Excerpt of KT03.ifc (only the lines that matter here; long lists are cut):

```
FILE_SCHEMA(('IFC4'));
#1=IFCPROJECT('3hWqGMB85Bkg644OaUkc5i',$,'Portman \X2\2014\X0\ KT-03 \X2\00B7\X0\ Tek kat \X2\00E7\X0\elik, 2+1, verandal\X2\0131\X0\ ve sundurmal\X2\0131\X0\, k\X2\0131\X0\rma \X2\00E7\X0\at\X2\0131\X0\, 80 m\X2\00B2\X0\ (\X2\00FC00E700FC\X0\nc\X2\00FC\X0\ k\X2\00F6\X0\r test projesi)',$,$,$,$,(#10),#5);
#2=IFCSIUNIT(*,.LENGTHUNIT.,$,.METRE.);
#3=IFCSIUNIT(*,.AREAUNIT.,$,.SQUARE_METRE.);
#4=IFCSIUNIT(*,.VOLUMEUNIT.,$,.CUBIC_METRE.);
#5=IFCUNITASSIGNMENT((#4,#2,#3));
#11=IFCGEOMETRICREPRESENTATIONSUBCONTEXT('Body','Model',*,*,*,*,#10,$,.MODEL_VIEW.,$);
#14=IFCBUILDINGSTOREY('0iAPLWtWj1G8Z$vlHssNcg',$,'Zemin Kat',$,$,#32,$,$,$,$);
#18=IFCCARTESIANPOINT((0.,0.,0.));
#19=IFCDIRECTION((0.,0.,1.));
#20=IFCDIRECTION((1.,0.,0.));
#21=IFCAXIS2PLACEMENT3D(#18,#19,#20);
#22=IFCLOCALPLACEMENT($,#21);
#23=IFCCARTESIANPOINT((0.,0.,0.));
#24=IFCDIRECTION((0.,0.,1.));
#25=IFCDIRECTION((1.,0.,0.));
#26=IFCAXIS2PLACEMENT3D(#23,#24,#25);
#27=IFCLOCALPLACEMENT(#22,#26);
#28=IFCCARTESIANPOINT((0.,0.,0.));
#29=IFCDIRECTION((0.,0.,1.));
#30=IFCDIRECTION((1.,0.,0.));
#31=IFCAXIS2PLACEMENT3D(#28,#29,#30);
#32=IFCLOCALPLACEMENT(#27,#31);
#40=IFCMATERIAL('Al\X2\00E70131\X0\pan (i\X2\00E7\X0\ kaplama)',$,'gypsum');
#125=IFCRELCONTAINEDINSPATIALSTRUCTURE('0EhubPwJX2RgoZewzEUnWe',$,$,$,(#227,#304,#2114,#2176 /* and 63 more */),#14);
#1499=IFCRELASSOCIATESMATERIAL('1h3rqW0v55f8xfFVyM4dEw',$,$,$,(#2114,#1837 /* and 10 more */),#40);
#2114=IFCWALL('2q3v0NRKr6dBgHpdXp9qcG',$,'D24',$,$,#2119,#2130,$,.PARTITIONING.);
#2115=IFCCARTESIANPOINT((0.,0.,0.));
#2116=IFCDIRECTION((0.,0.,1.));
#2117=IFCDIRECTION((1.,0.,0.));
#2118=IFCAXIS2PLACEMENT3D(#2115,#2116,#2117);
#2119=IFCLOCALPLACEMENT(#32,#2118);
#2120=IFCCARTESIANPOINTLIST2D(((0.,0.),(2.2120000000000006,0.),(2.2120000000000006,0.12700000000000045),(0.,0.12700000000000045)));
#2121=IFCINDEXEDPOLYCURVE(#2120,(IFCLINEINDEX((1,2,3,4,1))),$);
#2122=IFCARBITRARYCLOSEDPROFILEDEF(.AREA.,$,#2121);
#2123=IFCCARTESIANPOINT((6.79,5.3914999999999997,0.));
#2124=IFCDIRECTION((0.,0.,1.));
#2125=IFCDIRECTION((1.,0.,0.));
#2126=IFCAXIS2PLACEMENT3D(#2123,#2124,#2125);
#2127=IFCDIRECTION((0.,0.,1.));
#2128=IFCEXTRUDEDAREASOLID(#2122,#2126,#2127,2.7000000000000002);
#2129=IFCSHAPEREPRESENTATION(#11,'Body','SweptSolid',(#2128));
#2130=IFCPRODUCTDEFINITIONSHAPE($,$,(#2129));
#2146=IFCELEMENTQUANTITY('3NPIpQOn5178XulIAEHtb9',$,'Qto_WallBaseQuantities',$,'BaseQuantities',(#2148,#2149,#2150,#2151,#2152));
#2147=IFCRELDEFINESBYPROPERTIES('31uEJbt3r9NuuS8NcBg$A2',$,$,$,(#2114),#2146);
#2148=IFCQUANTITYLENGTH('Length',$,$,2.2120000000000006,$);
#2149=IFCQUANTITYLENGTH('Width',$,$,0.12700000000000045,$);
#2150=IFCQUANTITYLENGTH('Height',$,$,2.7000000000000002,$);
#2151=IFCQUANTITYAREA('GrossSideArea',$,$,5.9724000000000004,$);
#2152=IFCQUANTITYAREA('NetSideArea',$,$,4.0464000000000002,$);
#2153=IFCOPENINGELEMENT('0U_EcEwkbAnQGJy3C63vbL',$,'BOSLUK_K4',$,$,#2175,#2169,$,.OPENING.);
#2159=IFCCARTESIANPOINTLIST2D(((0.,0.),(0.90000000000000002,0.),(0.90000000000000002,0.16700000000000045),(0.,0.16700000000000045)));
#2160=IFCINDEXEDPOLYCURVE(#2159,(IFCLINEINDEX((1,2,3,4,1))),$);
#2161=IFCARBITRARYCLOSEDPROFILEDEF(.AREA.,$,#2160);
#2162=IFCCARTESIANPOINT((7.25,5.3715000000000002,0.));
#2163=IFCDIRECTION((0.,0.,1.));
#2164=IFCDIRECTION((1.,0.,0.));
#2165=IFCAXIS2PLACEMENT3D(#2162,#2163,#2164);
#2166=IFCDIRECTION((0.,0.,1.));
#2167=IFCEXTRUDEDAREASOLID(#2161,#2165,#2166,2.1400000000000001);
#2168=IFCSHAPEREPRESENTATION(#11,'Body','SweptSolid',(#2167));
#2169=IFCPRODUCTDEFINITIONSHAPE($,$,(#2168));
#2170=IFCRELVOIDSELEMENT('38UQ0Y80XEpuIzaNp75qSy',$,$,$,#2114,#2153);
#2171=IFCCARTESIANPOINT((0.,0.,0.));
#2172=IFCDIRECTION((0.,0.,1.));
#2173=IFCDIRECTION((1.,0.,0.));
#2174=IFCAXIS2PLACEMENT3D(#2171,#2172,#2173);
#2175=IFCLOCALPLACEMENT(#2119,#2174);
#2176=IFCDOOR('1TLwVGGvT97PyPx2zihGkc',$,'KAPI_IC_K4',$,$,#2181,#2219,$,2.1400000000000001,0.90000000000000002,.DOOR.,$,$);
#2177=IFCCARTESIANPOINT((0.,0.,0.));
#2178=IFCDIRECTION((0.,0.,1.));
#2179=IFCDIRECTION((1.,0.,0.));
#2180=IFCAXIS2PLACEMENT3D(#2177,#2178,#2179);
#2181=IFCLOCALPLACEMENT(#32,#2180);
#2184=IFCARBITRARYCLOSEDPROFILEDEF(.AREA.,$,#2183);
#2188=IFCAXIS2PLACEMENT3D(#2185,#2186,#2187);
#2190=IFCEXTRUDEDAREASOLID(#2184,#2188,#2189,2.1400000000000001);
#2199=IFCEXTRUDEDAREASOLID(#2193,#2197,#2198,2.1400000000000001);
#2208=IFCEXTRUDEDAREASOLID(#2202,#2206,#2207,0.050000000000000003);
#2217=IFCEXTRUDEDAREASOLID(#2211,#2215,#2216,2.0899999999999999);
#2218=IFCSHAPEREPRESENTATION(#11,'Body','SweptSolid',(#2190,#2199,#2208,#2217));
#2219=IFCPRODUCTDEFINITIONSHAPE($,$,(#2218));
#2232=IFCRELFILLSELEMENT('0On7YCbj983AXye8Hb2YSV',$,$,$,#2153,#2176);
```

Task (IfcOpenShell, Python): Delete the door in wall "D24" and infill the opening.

```python
import ifcopenshell
import ifcopenshell.api.feature
import ifcopenshell.api.pset
import ifcopenshell.api.root
import ifcopenshell.geom
import ifcopenshell.util.element
import ifcopenshell.util.shape
import ifcopenshell.util.unit

model = ifcopenshell.open("KT03.ifc")
area_scale = ifcopenshell.util.unit.calculate_unit_scale(model, "AREAUNIT")
settings = ifcopenshell.geom.settings()


def volume(element):
    """Net volume in cubic metres, openings subtracted."""
    shape = ifcopenshell.geom.create_shape(settings, element)
    return ifcopenshell.util.shape.get_volume(shape.geometry)


door = model.by_guid("1TLwVGGvT97PyPx2zihGkc")
opening = door.FillsVoids[0].RelatingOpeningElement
wall = opening.VoidsElements[0].RelatingBuildingElement
before = volume(wall)

ifcopenshell.api.root.remove_product(model, product=door)
ifcopenshell.api.feature.remove_feature(model, feature=opening)

after = volume(wall)
thickness = 0.127  # wall thickness in metres

# Update the wall's stored quantities.
qto = model.by_id(ifcopenshell.util.element.get_pset(wall, "Qto_WallBaseQuantities", should_inherit=False)["id"])
ifcopenshell.api.pset.edit_qto(model, qto=qto, properties={"NetSideArea": after / thickness / area_scale})

print(f"wall volume {before:.3f} -> {after:.3f} m3")

model.write("KT03_rev.ifc")
```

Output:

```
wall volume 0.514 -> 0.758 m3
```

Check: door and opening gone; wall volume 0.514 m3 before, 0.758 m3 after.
